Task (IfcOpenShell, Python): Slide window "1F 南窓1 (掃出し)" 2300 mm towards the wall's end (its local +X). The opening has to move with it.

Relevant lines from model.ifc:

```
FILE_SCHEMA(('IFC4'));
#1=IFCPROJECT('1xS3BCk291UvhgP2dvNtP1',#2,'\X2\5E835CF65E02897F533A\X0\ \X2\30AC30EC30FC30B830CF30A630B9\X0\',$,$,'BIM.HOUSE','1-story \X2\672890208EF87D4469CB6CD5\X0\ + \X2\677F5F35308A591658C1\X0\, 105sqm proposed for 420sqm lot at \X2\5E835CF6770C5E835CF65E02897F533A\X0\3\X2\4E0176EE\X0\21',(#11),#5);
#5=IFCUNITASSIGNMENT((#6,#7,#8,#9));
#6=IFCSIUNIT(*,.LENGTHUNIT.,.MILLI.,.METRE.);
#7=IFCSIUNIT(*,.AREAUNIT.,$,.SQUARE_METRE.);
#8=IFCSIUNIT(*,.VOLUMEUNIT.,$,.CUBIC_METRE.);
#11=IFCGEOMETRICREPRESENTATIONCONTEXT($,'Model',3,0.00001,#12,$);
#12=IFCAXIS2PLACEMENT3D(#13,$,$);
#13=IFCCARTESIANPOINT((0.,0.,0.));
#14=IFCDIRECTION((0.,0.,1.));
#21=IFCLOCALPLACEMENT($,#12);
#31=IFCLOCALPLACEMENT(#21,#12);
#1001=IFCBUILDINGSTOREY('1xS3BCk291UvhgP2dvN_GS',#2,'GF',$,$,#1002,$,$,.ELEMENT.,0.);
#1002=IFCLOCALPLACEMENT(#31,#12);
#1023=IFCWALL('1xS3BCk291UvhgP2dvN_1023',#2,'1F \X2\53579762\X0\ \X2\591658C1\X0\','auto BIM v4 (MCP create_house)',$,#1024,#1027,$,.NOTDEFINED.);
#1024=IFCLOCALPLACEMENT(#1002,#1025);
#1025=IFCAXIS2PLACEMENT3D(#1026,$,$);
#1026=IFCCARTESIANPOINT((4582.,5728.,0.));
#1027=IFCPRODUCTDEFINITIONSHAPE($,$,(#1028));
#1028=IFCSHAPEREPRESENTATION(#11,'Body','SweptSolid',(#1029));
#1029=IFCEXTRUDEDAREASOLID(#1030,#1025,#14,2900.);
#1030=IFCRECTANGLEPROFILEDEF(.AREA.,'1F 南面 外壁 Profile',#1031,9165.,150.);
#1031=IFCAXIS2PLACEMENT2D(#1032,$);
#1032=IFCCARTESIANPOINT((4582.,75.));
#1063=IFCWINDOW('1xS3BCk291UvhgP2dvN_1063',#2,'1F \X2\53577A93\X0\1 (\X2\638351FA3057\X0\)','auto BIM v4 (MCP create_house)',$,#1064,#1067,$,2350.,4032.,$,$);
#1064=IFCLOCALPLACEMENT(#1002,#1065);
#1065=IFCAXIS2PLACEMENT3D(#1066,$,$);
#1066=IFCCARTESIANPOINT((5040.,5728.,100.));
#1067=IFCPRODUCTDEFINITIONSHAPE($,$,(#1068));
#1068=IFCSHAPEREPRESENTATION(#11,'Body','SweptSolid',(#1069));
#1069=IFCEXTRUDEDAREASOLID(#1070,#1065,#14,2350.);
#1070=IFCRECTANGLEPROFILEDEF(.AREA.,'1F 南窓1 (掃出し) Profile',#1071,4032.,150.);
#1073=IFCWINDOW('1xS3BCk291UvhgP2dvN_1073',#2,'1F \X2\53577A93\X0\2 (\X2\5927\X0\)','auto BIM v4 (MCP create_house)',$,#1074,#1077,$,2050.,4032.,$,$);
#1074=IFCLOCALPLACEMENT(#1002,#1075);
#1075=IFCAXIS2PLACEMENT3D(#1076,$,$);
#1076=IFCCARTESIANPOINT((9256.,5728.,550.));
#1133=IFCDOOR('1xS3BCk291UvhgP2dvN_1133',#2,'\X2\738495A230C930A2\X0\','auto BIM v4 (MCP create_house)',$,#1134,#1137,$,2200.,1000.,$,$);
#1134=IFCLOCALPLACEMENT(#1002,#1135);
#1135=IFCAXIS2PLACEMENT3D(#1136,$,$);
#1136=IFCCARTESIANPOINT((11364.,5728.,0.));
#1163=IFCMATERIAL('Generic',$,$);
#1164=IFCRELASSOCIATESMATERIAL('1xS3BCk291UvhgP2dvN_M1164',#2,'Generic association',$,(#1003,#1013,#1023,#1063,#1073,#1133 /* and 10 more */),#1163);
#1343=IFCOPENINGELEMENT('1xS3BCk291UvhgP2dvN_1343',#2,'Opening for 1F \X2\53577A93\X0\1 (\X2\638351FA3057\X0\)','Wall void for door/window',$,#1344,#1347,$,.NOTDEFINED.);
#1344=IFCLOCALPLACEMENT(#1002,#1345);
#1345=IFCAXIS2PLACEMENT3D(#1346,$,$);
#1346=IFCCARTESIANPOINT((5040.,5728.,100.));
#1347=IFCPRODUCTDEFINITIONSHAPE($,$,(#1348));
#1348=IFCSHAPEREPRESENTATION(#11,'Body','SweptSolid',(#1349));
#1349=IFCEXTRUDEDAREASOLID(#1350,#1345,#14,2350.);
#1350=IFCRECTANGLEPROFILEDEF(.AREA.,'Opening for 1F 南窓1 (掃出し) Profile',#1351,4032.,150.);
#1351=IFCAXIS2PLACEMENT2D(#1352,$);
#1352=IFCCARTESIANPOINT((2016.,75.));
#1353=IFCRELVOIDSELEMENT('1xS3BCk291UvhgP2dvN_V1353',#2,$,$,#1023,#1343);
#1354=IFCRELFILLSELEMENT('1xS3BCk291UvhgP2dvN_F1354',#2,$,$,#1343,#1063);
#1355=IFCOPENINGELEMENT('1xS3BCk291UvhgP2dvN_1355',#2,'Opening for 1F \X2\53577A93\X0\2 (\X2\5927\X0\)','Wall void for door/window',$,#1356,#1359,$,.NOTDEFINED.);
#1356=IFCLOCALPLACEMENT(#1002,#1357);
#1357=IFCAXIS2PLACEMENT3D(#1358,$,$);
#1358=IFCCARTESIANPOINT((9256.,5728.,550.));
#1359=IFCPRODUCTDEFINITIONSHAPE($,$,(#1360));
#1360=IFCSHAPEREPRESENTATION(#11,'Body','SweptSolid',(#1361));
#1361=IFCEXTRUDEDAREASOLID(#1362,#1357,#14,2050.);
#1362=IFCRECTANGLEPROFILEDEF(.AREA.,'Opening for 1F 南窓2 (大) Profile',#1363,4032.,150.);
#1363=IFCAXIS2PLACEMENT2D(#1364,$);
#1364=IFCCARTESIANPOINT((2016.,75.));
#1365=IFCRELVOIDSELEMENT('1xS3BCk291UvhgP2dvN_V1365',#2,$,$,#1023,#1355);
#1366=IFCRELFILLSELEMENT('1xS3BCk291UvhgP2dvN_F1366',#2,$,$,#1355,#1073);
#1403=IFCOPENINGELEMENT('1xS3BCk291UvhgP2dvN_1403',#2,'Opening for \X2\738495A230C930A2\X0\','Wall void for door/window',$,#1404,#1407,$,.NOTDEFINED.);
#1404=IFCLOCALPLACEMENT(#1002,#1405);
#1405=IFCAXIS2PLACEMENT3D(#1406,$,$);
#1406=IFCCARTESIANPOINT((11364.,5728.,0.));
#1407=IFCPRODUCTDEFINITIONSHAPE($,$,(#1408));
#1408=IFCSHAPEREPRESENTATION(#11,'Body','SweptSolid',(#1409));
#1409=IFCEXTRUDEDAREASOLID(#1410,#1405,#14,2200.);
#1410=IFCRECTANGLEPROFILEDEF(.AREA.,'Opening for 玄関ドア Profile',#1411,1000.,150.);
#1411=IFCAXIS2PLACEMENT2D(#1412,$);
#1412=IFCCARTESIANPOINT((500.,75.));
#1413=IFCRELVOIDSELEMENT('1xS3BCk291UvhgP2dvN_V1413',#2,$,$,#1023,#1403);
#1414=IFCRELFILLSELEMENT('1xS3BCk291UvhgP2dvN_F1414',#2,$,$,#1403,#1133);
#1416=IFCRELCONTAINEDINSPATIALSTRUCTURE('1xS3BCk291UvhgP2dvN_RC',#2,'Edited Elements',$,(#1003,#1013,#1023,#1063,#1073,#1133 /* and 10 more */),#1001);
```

```python
import ifcopenshell
import ifcopenshell.api.geometry
import ifcopenshell.util.placement
import ifcopenshell.util.unit

model = ifcopenshell.open("model.ifc")
unit_scale = ifcopenshell.util.unit.calculate_unit_scale(model)

window = model.by_guid("1xS3BCk291UvhgP2dvN_1063")
opening = window.FillsVoids[0].RelatingOpeningElement
wall = opening.VoidsElements[0].RelatingBuildingElement

wall_matrix = ifcopenshell.util.placement.get_local_placement(wall.ObjectPlacement)
shift = wall_matrix[:3, 0] * 2.3 / unit_scale
before = ifcopenshell.util.placement.get_local_placement(window.ObjectPlacement)[:3, 3].copy()

# The window is not placed relative to its opening, so move both.
for product in (opening, window):
    matrix = ifcopenshell.util.placement.get_local_placement(product.ObjectPlacement)
    matrix[:3, 3] += shift
    ifcopenshell.api.geometry.edit_object_placement(model, product=product, matrix=matrix, is_si=False)

after = ifcopenshell.util.placement.get_local_placement(window.ObjectPlacement)[:3, 3]
print("window moved by", (after - before).round(3) + 0.0)

model.write("model_v2.ifc")
```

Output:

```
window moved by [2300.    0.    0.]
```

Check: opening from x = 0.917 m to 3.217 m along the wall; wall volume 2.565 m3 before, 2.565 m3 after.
